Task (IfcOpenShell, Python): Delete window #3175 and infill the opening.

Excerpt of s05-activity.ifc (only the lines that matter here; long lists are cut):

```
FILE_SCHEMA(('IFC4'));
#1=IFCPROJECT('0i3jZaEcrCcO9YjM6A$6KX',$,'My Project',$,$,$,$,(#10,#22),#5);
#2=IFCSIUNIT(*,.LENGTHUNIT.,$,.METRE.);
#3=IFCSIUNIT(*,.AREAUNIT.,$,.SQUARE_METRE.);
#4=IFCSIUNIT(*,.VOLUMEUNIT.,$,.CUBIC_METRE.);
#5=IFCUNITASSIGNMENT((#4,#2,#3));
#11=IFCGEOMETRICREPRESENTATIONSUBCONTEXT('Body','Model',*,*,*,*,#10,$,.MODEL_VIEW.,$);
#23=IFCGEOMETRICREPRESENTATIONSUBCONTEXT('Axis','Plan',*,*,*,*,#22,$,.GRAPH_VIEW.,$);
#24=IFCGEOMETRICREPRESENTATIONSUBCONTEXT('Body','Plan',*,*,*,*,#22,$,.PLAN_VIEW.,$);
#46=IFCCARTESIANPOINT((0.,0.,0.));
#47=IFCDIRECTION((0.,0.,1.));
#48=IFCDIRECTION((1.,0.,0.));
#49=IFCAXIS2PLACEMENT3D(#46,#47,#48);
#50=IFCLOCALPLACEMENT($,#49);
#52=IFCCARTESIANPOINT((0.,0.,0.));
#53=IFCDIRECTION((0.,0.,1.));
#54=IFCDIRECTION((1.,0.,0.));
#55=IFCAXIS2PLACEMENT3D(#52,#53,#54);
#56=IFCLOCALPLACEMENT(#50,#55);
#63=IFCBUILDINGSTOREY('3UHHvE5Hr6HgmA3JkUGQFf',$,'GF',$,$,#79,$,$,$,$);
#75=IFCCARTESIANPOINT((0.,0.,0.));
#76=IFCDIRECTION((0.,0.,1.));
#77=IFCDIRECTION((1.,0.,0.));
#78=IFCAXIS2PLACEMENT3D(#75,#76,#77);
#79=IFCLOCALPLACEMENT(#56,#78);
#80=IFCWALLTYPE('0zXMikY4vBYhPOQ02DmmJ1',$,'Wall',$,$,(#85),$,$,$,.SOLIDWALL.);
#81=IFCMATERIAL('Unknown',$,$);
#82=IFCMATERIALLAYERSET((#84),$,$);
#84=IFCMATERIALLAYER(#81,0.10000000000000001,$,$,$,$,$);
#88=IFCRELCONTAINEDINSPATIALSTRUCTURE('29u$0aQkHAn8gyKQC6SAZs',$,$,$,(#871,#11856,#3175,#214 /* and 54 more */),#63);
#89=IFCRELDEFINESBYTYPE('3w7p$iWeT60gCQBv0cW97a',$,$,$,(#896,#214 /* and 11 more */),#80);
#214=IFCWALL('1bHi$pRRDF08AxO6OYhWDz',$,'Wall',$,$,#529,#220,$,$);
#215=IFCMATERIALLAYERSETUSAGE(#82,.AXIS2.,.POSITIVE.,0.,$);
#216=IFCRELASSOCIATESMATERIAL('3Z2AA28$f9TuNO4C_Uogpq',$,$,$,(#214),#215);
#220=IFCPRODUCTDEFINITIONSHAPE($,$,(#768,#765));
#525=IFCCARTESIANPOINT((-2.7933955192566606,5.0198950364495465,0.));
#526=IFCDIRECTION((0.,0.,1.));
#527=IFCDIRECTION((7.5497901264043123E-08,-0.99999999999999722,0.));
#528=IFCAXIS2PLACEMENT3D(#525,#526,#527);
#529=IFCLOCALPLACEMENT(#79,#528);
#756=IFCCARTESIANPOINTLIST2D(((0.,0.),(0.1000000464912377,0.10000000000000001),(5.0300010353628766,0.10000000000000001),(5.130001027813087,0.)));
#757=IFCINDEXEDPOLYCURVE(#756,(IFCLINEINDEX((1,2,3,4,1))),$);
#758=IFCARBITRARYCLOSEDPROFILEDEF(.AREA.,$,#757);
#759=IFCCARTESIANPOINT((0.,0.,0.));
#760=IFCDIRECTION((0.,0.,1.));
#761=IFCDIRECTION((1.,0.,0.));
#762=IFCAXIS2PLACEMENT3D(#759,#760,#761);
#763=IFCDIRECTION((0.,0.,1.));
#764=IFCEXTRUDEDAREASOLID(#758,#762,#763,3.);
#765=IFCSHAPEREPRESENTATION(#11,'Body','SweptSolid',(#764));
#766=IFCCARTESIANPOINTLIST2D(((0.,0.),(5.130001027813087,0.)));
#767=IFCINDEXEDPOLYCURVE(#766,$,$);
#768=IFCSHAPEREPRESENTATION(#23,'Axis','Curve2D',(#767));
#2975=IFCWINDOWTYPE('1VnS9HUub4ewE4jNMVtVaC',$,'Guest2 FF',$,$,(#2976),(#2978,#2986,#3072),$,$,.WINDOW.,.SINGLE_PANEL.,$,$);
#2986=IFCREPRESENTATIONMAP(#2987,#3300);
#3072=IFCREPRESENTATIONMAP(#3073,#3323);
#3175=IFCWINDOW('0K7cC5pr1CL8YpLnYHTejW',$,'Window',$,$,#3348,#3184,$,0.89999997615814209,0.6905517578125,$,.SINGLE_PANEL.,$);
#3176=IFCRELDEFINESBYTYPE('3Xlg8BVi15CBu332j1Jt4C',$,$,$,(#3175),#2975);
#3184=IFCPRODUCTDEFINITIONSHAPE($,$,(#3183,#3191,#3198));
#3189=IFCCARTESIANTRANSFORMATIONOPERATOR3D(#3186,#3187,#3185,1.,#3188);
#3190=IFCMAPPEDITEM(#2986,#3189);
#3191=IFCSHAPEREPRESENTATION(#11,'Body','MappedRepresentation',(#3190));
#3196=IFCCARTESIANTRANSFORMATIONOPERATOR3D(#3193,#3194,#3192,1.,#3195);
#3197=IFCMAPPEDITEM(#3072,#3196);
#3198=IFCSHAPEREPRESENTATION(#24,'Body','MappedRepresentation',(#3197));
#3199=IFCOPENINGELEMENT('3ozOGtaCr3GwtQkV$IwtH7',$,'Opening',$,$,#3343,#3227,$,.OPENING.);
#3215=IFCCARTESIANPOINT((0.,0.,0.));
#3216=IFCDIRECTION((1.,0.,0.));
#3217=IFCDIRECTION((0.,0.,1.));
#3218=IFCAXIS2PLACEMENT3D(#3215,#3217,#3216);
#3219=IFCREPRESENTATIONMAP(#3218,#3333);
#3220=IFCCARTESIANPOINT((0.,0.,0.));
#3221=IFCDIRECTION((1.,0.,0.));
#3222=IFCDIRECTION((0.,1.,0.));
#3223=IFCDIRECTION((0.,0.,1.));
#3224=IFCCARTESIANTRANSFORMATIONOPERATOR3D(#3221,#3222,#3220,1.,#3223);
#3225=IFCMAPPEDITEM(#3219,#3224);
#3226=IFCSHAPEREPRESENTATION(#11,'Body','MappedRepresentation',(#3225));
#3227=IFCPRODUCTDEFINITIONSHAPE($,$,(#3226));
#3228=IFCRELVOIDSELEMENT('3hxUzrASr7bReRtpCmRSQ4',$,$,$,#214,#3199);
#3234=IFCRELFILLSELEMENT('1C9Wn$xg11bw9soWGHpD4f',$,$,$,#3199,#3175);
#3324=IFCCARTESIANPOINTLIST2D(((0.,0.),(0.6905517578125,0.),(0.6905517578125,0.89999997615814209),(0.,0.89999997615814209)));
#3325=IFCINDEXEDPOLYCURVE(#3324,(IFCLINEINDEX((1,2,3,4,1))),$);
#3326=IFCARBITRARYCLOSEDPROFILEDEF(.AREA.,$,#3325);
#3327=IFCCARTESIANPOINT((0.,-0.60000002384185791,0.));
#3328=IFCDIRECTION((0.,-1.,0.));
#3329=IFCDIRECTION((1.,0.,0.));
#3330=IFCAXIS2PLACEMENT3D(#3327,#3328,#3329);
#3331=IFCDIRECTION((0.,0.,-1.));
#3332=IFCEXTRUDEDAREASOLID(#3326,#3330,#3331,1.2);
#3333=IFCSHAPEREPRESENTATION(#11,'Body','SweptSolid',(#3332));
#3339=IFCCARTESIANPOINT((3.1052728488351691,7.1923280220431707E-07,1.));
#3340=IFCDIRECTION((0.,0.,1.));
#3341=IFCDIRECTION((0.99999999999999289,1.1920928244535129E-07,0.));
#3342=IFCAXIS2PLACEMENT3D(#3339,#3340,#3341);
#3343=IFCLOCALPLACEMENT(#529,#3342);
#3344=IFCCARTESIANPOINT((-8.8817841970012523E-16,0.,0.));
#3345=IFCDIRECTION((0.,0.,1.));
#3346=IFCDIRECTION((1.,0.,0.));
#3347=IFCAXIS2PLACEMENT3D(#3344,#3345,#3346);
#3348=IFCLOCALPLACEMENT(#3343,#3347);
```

```python
import ifcopenshell
import ifcopenshell.api.feature
import ifcopenshell.api.root
import ifcopenshell.geom
import ifcopenshell.util.shape

model = ifcopenshell.open("s05-activity.ifc")
settings = ifcopenshell.geom.settings()


def volume(element):
    """Net volume in cubic metres, openings subtracted."""
    shape = ifcopenshell.geom.create_shape(settings, element)
    return ifcopenshell.util.shape.get_volume(shape.geometry)


window = model.by_id(3175)
opening = window.FillsVoids[0].RelatingOpeningElement
wall = opening.VoidsElements[0].RelatingBuildingElement
before = volume(wall)

ifcopenshell.api.root.remove_product(model, product=window)
ifcopenshell.api.feature.remove_feature(model, feature=opening)

after = volume(wall)

print(f"wall volume {before:.3f} -> {after:.3f} m3")

model.write("s05-activity-out.ifc")
```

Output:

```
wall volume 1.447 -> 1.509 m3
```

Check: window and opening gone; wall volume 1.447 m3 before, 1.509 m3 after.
